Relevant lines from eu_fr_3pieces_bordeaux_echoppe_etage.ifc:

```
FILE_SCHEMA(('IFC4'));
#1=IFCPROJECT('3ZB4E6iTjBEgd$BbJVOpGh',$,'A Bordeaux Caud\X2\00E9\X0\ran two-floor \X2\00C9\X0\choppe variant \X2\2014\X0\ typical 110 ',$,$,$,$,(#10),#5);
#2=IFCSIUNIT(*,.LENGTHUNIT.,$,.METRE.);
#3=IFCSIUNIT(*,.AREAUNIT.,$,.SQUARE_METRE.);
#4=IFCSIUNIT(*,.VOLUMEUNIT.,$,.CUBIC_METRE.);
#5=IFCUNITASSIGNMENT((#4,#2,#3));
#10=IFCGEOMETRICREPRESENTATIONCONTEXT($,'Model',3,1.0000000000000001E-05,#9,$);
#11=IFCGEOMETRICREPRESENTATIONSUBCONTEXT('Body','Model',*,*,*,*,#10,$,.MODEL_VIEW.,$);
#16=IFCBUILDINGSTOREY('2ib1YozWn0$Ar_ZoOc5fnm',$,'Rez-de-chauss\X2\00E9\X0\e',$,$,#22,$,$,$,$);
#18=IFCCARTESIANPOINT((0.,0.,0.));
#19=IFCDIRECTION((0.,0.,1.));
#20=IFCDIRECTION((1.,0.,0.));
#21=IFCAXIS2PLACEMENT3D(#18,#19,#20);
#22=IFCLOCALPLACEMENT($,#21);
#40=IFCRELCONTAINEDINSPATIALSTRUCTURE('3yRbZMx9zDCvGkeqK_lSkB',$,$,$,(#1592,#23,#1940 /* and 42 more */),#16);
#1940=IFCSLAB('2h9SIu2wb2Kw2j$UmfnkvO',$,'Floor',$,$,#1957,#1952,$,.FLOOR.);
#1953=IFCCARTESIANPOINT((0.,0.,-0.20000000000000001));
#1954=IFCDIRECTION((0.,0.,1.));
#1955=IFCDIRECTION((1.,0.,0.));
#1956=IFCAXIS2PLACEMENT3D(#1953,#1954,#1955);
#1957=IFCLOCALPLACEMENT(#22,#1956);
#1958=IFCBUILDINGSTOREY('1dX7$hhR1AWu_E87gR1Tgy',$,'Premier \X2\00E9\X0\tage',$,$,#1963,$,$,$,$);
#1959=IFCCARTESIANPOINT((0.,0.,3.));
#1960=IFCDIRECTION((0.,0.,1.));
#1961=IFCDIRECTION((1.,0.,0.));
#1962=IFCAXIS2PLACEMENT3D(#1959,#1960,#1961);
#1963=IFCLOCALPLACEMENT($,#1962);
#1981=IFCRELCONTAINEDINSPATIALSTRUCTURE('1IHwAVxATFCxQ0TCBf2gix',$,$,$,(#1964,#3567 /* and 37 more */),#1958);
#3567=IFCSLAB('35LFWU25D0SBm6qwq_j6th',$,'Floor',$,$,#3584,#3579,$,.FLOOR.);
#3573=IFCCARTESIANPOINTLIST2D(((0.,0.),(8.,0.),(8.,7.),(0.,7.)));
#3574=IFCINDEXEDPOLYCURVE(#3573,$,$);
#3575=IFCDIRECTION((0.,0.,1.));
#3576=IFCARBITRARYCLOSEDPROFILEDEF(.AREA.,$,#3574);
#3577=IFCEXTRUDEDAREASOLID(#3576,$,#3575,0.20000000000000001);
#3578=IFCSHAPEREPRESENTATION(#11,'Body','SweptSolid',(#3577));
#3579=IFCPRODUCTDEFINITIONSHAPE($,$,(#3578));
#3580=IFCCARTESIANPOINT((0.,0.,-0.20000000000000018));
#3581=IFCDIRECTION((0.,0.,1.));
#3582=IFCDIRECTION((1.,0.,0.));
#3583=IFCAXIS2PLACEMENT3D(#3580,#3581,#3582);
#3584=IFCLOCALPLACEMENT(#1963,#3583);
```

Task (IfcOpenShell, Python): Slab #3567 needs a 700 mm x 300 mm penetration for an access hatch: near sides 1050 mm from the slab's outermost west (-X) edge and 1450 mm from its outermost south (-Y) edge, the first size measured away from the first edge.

```python
import numpy as np
import ifcopenshell
import ifcopenshell.api.feature
import ifcopenshell.api.geometry
import ifcopenshell.api.root
import ifcopenshell.geom
import ifcopenshell.util.placement
import ifcopenshell.util.representation
import ifcopenshell.util.shape
import ifcopenshell.util.unit

model = ifcopenshell.open("eu_fr_3pieces_bordeaux_echoppe_etage.ifc")
unit_scale = ifcopenshell.util.unit.calculate_unit_scale(model)
settings = ifcopenshell.geom.settings()


def volume(element):
    """Net volume in cubic metres, openings subtracted."""
    shape = ifcopenshell.geom.create_shape(settings, element)
    return ifcopenshell.util.shape.get_volume(shape.geometry)


slab = model.by_id(3567)
before = volume(slab)

# Extent in the slab's own axes, in metres. The edges named are its -X and -Y sides.
slab_shape = ifcopenshell.geom.create_shape(settings, slab)
vertices = ifcopenshell.util.shape.get_vertices(slab_shape.geometry)
x_min, y_min, bottom = vertices.min(axis=0)
top = vertices[:, 2].max()

opening = ifcopenshell.api.root.create_entity(model, ifc_class="IfcOpeningElement", name="Access hatch opening", predefined_type="OPENING")
context = ifcopenshell.util.representation.get_context(model, "Model", "Body", "MODEL_VIEW")
width, depth = 0.7, 0.3
outline = [(0.0, 0.0), (width, 0.0), (width, depth), (0.0, depth), (0.0, 0.0)]
# Overshoot both faces by 50 mm so the cut is clean.
shape = ifcopenshell.api.geometry.add_slab_representation(
    model, context=context, depth=top - bottom + 0.1, polyline=outline
)
ifcopenshell.api.geometry.assign_representation(model, product=opening, representation=shape)

matrix = ifcopenshell.util.placement.get_local_placement(slab.ObjectPlacement)
matrix[:, 3] = matrix @ np.append(np.array([x_min + 1.05, y_min + 1.45, bottom - 0.05]) / unit_scale, 1.0)
ifcopenshell.api.geometry.edit_object_placement(model, product=opening, matrix=matrix, is_si=False)
ifcopenshell.api.feature.add_feature(model, feature=opening, element=slab)

after = volume(slab)

print(f"slab volume {before:.3f} -> {after:.3f} m3")

model.write("eu_fr_3pieces_bordeaux_echoppe_etage_updated.ifc")
```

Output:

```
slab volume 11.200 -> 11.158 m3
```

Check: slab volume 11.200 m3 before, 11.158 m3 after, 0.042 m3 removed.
